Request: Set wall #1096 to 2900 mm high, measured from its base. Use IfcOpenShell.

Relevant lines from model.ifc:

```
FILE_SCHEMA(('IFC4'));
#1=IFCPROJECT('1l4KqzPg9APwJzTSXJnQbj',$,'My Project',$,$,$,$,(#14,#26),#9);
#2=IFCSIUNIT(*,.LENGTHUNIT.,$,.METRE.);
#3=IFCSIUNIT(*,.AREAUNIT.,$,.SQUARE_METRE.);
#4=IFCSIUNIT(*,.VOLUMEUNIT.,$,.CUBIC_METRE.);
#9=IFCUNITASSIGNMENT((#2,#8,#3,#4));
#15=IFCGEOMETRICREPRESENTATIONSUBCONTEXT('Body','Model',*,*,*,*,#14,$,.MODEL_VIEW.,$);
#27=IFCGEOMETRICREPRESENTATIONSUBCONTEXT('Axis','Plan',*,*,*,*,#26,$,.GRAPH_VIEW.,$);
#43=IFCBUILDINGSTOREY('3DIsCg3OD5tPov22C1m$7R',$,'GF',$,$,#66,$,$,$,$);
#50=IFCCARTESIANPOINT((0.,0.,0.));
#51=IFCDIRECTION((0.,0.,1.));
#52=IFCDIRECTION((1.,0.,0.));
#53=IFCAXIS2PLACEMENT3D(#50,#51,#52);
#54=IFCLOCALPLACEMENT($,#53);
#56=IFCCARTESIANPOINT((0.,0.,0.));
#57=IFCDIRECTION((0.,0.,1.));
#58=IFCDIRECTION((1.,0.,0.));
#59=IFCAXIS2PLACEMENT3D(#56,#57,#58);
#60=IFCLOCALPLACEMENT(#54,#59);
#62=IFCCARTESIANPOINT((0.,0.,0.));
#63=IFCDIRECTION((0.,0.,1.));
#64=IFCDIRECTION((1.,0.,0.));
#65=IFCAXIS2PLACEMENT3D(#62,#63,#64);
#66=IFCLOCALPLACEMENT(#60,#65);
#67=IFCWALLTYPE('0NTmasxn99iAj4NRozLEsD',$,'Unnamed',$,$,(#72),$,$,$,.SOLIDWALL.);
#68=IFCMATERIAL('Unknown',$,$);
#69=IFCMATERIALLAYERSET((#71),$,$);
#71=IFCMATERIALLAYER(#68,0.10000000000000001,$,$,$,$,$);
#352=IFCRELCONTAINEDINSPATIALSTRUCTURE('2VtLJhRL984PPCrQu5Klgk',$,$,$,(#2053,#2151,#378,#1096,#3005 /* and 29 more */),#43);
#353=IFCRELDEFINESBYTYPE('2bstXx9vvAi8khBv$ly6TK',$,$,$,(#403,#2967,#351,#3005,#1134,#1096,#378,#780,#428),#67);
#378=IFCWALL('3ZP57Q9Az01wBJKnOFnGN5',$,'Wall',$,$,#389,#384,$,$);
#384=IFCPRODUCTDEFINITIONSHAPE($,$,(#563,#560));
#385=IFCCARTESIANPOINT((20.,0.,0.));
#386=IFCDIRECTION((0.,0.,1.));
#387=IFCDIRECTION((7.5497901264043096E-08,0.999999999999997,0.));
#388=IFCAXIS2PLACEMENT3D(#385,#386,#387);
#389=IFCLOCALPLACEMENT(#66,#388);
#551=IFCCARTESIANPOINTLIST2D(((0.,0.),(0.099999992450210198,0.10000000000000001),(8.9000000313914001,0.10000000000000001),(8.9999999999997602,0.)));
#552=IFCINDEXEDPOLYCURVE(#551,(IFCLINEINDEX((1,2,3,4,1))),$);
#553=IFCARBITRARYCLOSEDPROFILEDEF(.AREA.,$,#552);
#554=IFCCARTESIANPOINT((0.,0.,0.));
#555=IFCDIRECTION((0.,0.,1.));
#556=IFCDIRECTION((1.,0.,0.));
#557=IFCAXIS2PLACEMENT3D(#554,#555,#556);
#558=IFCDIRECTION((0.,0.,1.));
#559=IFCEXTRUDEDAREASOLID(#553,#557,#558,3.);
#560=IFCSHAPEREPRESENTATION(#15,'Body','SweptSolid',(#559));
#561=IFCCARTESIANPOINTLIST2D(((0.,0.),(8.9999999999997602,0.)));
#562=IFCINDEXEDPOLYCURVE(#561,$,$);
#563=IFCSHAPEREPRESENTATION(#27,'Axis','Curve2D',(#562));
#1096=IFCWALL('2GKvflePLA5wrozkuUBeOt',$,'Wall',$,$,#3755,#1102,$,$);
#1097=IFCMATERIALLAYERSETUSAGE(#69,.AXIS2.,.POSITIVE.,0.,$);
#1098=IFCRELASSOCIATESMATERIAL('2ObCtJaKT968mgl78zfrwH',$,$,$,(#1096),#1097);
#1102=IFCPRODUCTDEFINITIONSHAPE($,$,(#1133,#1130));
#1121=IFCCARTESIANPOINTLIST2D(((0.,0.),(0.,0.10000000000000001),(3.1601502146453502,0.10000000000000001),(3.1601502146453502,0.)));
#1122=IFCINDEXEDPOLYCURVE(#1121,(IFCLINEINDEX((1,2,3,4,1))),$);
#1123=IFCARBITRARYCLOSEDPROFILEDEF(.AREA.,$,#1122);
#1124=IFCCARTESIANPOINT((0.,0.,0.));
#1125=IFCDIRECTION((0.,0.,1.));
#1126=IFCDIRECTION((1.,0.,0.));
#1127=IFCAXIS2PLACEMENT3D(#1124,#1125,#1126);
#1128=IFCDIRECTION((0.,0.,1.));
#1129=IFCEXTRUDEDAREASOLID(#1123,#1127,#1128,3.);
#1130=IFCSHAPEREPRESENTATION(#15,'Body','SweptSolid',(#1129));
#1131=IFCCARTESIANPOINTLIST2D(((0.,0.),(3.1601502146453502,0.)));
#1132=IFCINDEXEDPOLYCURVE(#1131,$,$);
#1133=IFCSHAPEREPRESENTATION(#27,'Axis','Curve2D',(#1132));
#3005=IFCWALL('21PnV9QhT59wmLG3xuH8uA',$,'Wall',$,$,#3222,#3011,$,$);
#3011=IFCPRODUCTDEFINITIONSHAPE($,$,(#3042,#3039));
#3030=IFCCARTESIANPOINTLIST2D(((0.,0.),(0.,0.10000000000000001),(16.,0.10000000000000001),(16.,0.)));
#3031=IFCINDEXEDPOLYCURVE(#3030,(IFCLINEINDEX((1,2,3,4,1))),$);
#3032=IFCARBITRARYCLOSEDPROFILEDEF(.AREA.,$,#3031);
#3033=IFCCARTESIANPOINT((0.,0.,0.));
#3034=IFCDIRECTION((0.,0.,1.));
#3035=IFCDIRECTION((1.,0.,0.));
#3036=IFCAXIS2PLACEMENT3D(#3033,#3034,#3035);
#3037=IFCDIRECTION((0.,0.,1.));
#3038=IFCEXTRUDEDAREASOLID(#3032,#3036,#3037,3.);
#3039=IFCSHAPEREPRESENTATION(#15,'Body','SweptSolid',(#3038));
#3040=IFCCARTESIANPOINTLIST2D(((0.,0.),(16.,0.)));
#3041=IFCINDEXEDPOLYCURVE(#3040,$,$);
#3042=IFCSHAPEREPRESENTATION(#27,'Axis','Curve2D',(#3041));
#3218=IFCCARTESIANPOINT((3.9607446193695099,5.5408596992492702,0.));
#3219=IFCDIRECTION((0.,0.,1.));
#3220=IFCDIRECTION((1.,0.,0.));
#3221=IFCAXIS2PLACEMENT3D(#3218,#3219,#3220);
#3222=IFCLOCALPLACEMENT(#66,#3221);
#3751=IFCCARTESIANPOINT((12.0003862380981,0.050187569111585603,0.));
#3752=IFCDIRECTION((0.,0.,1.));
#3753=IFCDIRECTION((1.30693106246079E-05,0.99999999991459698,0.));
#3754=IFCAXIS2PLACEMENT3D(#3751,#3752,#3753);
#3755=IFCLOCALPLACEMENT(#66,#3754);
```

```python
import ifcopenshell
import ifcopenshell.geom
import ifcopenshell.util.representation
import ifcopenshell.util.shape

model = ifcopenshell.open("model.ifc")
settings = ifcopenshell.geom.settings()


def volume(element):
    """Net volume in cubic metres, openings subtracted."""
    shape = ifcopenshell.geom.create_shape(settings, element)
    return ifcopenshell.util.shape.get_volume(shape.geometry)


wall = model.by_guid("2GKvflePLA5wrozkuUBeOt")
before = volume(wall)

body = ifcopenshell.util.representation.get_representation(wall, "Model", "Body")
solid = body.Items[0]
old_height = solid.Depth
solid.Depth = 2.9
after = volume(wall)

print(f"height {old_height:g} -> {solid.Depth:g}, volume {before:.3f} -> {after:.3f} m3")

model.write("model_edited.ifc")
```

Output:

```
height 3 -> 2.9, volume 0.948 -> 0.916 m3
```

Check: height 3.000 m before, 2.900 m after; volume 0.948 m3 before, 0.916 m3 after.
